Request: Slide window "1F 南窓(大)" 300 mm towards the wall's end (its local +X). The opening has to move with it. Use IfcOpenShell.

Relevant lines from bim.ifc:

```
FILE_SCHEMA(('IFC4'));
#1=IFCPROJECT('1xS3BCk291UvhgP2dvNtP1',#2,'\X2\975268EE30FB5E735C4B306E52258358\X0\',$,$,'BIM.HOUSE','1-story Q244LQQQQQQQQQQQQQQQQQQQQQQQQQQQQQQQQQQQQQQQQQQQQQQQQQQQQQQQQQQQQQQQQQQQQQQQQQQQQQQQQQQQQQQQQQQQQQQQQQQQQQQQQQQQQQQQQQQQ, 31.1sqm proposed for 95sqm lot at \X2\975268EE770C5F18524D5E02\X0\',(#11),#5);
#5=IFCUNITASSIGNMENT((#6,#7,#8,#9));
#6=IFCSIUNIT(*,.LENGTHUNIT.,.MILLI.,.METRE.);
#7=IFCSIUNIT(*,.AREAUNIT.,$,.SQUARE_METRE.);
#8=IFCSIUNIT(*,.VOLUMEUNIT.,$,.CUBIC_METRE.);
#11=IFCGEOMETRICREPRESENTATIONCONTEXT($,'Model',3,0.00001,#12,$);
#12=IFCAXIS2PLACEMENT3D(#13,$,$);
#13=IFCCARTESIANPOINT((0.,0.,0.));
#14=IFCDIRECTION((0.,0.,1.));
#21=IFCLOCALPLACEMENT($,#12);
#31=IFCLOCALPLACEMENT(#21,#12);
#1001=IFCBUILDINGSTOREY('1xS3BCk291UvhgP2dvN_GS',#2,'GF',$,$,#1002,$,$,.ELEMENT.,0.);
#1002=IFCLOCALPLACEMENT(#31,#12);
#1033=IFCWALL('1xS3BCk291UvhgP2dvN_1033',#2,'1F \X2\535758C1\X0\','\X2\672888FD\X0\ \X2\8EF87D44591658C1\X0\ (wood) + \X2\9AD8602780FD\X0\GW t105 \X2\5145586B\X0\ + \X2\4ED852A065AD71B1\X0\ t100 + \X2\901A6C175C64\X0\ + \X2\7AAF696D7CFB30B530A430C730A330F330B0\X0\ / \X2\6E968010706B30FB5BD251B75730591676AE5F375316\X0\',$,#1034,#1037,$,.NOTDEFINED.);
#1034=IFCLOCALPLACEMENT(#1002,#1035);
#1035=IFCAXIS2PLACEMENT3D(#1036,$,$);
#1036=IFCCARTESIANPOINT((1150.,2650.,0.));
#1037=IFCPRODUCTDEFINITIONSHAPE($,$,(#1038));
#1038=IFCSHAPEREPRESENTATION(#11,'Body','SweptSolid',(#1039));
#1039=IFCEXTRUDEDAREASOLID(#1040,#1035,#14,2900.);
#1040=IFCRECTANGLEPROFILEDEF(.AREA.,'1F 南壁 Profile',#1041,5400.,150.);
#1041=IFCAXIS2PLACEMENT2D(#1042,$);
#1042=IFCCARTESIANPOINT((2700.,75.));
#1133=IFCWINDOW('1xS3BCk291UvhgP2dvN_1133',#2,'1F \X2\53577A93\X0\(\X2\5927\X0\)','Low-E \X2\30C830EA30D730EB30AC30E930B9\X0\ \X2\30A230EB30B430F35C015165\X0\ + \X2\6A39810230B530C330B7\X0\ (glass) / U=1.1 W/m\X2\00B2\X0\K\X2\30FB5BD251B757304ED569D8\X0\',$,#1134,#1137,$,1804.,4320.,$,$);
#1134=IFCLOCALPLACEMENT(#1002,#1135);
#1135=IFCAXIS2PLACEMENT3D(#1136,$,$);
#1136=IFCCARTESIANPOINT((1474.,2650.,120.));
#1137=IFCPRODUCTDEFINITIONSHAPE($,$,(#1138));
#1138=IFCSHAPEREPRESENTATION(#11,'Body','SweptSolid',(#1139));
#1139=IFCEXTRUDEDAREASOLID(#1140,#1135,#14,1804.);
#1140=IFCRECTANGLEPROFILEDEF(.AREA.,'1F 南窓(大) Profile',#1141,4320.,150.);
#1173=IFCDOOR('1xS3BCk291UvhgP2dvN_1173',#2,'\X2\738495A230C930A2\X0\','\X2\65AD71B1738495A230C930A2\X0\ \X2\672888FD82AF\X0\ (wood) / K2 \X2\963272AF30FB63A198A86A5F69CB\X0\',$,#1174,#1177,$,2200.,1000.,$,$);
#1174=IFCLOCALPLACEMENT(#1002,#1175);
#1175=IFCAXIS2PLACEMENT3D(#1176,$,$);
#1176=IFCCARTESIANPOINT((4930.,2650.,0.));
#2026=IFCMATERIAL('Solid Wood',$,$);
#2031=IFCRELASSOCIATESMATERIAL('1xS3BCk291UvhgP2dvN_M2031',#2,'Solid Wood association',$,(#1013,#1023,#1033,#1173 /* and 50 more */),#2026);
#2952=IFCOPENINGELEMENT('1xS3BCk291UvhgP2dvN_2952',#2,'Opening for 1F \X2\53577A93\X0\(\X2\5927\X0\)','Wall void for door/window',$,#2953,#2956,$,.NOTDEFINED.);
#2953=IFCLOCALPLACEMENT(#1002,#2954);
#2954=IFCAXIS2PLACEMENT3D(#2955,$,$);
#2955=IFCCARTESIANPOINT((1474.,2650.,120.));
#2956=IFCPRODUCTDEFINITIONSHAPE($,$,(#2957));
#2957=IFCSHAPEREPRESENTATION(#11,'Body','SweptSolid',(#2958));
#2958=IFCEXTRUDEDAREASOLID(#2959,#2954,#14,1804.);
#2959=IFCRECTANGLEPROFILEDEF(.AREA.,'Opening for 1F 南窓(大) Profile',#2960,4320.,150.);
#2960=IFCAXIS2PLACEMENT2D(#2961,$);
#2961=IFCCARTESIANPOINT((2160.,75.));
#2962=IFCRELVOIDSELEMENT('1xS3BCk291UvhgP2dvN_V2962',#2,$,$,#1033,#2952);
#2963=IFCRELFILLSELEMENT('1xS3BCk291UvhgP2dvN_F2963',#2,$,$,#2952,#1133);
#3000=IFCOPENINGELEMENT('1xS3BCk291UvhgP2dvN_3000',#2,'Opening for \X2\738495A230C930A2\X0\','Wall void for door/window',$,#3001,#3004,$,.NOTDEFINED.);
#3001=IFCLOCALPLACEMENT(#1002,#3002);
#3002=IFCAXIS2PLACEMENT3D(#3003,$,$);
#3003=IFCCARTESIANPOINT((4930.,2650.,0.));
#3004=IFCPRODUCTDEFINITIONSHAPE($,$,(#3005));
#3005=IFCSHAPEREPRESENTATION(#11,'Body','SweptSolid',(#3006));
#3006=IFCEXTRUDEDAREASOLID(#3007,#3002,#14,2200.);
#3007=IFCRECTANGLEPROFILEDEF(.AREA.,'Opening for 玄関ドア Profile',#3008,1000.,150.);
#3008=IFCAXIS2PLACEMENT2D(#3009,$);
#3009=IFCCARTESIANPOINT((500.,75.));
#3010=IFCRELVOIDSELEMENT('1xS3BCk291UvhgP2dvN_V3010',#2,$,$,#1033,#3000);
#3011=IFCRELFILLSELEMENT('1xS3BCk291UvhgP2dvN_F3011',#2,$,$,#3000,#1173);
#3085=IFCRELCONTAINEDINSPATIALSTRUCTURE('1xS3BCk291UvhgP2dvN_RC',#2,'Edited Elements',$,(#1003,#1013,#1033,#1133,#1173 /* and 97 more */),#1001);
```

```python
import ifcopenshell
import ifcopenshell.api.geometry
import ifcopenshell.util.placement
import ifcopenshell.util.unit

model = ifcopenshell.open("bim.ifc")
unit_scale = ifcopenshell.util.unit.calculate_unit_scale(model)

window = model.by_guid("1xS3BCk291UvhgP2dvN_1133")
opening = window.FillsVoids[0].RelatingOpeningElement
wall = opening.VoidsElements[0].RelatingBuildingElement

wall_matrix = ifcopenshell.util.placement.get_local_placement(wall.ObjectPlacement)
shift = wall_matrix[:3, 0] * 0.3 / unit_scale
before = ifcopenshell.util.placement.get_local_placement(window.ObjectPlacement)[:3, 3].copy()

# The window is not placed relative to its opening, so move both.
for product in (opening, window):
    matrix = ifcopenshell.util.placement.get_local_placement(product.ObjectPlacement)
    matrix[:3, 3] += shift
    ifcopenshell.api.geometry.edit_object_placement(model, product=product, matrix=matrix, is_si=False)

after = ifcopenshell.util.placement.get_local_placement(window.ObjectPlacement)[:3, 3]
print("window moved by", (after - before).round(3) + 0.0)

model.write("bim_v2.ifc")
```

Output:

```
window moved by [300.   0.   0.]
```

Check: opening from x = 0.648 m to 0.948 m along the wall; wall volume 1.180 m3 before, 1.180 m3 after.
